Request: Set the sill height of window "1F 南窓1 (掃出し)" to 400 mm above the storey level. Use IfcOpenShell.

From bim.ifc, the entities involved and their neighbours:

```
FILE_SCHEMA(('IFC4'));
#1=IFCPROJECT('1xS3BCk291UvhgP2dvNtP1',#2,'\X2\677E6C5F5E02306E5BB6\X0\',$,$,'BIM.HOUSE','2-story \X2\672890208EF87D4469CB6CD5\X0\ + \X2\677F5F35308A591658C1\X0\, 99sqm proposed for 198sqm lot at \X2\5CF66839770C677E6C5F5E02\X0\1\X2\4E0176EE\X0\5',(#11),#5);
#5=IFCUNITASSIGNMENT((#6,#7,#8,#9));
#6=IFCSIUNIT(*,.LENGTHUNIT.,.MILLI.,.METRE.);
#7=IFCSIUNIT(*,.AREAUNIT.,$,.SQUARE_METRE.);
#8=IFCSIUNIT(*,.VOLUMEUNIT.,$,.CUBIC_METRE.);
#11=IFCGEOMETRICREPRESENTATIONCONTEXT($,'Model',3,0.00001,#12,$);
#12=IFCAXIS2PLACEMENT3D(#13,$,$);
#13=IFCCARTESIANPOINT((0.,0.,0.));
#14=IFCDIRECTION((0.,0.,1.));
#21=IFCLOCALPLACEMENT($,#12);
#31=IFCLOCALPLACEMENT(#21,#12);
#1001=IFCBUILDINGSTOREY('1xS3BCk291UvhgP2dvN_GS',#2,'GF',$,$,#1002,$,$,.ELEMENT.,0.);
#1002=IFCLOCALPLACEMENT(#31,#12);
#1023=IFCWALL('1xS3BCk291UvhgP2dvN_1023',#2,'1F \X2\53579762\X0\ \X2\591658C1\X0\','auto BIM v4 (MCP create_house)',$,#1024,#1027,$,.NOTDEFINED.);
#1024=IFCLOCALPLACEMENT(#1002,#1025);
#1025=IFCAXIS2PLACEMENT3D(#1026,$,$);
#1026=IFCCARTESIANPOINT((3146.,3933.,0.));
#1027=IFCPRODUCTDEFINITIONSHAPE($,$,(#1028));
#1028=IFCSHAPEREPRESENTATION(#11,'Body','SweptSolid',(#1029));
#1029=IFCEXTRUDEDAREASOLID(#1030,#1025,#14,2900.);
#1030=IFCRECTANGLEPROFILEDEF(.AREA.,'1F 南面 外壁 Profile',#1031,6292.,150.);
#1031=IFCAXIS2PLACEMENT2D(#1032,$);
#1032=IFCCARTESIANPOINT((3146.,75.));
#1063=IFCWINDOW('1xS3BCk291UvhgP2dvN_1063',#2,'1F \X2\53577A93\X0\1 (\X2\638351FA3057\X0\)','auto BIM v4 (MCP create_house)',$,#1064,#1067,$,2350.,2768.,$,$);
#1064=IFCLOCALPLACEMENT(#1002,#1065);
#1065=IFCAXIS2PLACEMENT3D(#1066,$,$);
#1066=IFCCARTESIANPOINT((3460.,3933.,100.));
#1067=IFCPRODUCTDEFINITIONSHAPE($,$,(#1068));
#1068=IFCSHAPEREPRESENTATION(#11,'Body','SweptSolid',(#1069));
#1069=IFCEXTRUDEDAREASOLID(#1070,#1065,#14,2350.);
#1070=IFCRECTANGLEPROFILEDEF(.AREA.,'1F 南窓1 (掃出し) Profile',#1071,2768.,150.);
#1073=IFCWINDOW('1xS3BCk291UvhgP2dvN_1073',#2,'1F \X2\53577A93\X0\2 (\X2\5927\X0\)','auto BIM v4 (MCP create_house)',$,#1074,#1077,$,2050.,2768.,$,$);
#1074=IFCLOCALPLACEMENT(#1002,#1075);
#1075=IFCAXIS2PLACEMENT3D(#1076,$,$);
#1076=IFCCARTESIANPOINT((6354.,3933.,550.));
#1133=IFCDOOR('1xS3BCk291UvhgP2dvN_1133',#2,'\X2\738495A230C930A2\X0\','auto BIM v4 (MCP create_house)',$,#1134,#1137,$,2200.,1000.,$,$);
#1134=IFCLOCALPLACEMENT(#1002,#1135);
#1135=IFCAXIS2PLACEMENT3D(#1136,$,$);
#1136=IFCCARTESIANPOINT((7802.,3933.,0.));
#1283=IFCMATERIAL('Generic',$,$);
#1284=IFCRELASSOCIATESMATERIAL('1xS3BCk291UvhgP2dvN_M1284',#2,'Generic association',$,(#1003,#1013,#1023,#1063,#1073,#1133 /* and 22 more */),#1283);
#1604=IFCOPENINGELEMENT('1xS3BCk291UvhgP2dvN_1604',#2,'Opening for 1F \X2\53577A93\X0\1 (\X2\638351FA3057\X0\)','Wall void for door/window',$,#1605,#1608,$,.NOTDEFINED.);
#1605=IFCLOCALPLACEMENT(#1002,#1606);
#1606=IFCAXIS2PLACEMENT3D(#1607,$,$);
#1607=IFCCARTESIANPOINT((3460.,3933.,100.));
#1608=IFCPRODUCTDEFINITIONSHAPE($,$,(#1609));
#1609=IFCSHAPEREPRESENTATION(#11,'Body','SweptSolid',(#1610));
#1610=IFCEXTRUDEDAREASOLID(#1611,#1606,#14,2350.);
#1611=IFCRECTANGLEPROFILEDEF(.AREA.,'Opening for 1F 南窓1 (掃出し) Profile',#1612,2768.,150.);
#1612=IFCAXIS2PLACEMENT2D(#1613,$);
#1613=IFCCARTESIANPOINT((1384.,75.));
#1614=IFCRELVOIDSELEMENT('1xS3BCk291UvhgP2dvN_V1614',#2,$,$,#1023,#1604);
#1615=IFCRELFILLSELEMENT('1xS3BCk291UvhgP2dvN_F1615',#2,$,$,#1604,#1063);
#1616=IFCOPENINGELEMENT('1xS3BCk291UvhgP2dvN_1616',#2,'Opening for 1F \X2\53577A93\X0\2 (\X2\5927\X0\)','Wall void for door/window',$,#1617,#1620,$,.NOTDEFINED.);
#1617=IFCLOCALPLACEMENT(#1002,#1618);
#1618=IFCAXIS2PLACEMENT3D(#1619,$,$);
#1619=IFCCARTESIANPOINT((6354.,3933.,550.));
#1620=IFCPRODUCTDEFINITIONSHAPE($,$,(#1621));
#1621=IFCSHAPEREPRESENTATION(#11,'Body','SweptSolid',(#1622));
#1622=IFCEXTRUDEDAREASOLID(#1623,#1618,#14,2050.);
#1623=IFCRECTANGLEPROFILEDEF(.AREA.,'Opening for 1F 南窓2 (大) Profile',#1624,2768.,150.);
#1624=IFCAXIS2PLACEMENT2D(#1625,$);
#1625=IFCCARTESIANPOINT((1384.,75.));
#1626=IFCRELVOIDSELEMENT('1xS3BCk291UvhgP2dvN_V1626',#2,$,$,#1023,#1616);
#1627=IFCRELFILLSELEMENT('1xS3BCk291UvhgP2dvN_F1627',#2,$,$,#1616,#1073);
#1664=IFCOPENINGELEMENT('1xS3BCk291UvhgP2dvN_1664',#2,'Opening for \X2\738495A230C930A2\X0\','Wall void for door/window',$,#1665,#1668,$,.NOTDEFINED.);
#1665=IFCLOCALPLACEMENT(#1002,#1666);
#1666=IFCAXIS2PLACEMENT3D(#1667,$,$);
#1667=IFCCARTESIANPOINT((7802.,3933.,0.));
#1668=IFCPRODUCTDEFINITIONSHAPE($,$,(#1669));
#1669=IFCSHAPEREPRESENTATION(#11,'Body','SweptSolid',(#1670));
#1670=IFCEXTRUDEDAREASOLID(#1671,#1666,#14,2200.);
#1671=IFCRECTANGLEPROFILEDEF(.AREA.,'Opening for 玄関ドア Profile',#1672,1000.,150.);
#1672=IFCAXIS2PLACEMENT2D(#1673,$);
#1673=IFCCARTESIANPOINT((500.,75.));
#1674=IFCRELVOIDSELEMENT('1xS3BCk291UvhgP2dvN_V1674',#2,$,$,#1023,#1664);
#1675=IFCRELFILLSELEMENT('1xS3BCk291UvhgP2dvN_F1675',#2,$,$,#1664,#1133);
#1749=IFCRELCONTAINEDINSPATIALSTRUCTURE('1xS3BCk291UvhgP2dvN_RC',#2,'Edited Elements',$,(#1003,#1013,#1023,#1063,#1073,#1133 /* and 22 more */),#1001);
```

```python
import numpy as np
import ifcopenshell
import ifcopenshell.api.geometry
import ifcopenshell.geom
import ifcopenshell.util.element
import ifcopenshell.util.placement
import ifcopenshell.util.shape
import ifcopenshell.util.unit

model = ifcopenshell.open("bim.ifc")
unit_scale = ifcopenshell.util.unit.calculate_unit_scale(model)

window = model.by_guid("1xS3BCk291UvhgP2dvN_1063")
opening = window.FillsVoids[0].RelatingOpeningElement
storey = ifcopenshell.util.element.get_container(window, ifc_class="IfcBuildingStorey")
level = ifcopenshell.util.placement.get_local_placement(storey.ObjectPlacement)[2, 3]

# The opening's origin need not be at the sill, so measure its lowest point.
shape = ifcopenshell.geom.create_shape(ifcopenshell.geom.settings(), opening)
bottom = ifcopenshell.util.shape.get_shape_bottom_elevation(shape, shape.geometry) / unit_scale
dz = level + 0.4 / unit_scale - bottom

shift = np.array([0.0, 0.0, dz])
# The window is not placed relative to its opening, so move both.
for product in (opening, window):
    matrix = ifcopenshell.util.placement.get_local_placement(product.ObjectPlacement)
    matrix[:3, 3] += shift
    ifcopenshell.api.geometry.edit_object_placement(model, product=product, matrix=matrix, is_si=False)

print(f"moved by {dz * unit_scale:+.3f} m")

model.write("bim_updated.ifc")
```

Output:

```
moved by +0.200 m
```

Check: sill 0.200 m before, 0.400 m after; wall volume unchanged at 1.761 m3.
